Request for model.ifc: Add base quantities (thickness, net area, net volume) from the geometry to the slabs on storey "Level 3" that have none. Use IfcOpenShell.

First a look at what the model holds.

```python
import ifcopenshell
import ifcopenshell.util.element
import ifcopenshell.util.unit

model = ifcopenshell.open("model.ifc")
print(model.schema)
for unit_type in ("LENGTHUNIT", "AREAUNIT", "VOLUMEUNIT"):
    print(unit_type, ifcopenshell.util.unit.calculate_unit_scale(model, unit_type))
storey = next(s for s in model.by_type("IfcBuildingStorey") if s.Name == "Level 3")
slabs = [e for e in ifcopenshell.util.element.get_decomposition(storey) if e.is_a("IfcSlab")]
for e in sorted(slabs, key=lambda e: e.id()):
    print(e.id(), e.is_a(), e.Name, list(ifcopenshell.util.element.get_psets(e, qtos_only=True)), sep=" | ")
```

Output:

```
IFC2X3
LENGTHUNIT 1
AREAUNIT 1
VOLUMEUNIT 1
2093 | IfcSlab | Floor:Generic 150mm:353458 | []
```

```python
import ifcopenshell
import ifcopenshell.api.pset
import ifcopenshell.geom
import ifcopenshell.util.element
import ifcopenshell.util.shape
import ifcopenshell.util.unit

model = ifcopenshell.open("model.ifc")
unit_scale = ifcopenshell.util.unit.calculate_unit_scale(model)
area_scale = ifcopenshell.util.unit.calculate_unit_scale(model, "AREAUNIT")
volume_scale = ifcopenshell.util.unit.calculate_unit_scale(model, "VOLUMEUNIT")
settings = ifcopenshell.geom.settings()

storey = next(s for s in model.by_type("IfcBuildingStorey") if s.Name == "Level 3")
slabs = [e for e in ifcopenshell.util.element.get_decomposition(storey) if e.is_a("IfcSlab")]

for e in sorted(slabs, key=lambda e: e.id()):
    if ifcopenshell.util.element.get_psets(e, qtos_only=True, should_inherit=False):
        continue
    # Geometry comes back in metres, in the element's own axes.
    shape = ifcopenshell.geom.create_shape(settings, e)
    values = {
        "Width": ifcopenshell.util.shape.get_z(shape.geometry) / unit_scale,
        "NetArea": ifcopenshell.util.shape.get_footprint_area(shape.geometry) / area_scale,
        "NetVolume": ifcopenshell.util.shape.get_volume(shape.geometry) / volume_scale,
    }
    qto = ifcopenshell.api.pset.add_qto(model, product=e, name="BaseQuantities")
    ifcopenshell.api.pset.edit_qto(model, qto=qto, properties=values)
    print(e.id(), {k: round(v, 3) for k, v in values.items()})

model.write("model_edited.ifc")
```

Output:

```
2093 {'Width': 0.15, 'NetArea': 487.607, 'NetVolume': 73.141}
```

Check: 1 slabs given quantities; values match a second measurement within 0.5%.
